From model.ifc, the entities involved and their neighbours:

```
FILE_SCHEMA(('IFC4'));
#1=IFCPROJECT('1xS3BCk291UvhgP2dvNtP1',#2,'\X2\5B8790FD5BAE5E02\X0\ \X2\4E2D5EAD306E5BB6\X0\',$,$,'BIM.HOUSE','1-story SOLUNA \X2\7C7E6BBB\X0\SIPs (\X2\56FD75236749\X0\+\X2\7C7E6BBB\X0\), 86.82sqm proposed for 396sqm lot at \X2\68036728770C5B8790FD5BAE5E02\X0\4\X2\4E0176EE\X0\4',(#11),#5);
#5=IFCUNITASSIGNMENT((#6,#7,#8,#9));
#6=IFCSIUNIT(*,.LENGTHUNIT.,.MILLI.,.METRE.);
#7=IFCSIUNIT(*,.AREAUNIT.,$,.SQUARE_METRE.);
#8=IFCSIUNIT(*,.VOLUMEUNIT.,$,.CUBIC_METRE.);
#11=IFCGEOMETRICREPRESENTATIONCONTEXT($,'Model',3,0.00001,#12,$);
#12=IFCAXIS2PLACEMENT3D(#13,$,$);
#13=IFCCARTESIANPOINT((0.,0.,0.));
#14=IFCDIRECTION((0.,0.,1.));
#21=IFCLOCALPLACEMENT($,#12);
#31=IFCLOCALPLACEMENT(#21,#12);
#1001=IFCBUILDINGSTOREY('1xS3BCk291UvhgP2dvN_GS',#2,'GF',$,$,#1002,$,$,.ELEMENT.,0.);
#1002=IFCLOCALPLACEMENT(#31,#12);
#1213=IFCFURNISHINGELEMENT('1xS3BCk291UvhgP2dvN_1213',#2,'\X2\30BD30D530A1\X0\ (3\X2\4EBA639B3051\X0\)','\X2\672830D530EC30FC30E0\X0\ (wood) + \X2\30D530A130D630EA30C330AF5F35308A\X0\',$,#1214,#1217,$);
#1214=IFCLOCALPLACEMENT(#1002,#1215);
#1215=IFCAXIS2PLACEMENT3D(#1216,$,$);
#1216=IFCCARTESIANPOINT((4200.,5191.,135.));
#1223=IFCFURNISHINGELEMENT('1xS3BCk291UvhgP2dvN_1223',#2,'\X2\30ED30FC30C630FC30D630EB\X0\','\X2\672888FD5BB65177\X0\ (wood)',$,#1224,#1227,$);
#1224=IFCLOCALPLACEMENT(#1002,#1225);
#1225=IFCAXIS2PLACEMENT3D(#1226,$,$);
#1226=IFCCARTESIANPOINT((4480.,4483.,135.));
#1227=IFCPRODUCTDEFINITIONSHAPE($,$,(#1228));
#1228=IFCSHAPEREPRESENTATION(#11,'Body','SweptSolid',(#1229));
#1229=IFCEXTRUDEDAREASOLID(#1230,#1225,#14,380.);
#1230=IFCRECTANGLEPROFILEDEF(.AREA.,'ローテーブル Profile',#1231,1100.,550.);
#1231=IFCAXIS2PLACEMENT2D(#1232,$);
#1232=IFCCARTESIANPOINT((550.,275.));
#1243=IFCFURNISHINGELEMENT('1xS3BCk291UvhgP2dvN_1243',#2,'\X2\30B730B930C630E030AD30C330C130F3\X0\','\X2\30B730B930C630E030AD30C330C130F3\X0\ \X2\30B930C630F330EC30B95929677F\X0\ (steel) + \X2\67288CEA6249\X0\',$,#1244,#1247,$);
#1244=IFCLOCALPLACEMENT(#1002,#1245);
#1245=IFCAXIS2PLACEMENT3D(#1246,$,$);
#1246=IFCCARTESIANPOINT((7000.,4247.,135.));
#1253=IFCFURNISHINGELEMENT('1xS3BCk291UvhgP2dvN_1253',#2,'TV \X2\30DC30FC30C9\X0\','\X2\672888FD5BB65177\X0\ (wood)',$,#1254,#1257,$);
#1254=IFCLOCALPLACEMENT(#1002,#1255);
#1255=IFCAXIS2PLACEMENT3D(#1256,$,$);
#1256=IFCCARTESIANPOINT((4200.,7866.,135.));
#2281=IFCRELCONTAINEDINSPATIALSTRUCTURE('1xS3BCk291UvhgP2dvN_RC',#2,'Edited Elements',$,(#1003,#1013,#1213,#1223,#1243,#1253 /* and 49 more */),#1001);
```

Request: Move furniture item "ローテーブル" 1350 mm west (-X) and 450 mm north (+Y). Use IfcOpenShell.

```python
import ifcopenshell
import ifcopenshell.api.geometry
import ifcopenshell.util.placement
import ifcopenshell.util.unit

model = ifcopenshell.open("model.ifc")
unit_scale = ifcopenshell.util.unit.calculate_unit_scale(model)

item = model.by_guid("1xS3BCk291UvhgP2dvN_1223")
matrix = ifcopenshell.util.placement.get_local_placement(item.ObjectPlacement)
matrix[0, 3] -= 1.35 / unit_scale
matrix[1, 3] += 0.45 / unit_scale
ifcopenshell.api.geometry.edit_object_placement(model, product=item, matrix=matrix, is_si=False)

print(ifcopenshell.util.placement.get_local_placement(item.ObjectPlacement).round(3) + 0.0)

model.write("model_updated.ifc")
```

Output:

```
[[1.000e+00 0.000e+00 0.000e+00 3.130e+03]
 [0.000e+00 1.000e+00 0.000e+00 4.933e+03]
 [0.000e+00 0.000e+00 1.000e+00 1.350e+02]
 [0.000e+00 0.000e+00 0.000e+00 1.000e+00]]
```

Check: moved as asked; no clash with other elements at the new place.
